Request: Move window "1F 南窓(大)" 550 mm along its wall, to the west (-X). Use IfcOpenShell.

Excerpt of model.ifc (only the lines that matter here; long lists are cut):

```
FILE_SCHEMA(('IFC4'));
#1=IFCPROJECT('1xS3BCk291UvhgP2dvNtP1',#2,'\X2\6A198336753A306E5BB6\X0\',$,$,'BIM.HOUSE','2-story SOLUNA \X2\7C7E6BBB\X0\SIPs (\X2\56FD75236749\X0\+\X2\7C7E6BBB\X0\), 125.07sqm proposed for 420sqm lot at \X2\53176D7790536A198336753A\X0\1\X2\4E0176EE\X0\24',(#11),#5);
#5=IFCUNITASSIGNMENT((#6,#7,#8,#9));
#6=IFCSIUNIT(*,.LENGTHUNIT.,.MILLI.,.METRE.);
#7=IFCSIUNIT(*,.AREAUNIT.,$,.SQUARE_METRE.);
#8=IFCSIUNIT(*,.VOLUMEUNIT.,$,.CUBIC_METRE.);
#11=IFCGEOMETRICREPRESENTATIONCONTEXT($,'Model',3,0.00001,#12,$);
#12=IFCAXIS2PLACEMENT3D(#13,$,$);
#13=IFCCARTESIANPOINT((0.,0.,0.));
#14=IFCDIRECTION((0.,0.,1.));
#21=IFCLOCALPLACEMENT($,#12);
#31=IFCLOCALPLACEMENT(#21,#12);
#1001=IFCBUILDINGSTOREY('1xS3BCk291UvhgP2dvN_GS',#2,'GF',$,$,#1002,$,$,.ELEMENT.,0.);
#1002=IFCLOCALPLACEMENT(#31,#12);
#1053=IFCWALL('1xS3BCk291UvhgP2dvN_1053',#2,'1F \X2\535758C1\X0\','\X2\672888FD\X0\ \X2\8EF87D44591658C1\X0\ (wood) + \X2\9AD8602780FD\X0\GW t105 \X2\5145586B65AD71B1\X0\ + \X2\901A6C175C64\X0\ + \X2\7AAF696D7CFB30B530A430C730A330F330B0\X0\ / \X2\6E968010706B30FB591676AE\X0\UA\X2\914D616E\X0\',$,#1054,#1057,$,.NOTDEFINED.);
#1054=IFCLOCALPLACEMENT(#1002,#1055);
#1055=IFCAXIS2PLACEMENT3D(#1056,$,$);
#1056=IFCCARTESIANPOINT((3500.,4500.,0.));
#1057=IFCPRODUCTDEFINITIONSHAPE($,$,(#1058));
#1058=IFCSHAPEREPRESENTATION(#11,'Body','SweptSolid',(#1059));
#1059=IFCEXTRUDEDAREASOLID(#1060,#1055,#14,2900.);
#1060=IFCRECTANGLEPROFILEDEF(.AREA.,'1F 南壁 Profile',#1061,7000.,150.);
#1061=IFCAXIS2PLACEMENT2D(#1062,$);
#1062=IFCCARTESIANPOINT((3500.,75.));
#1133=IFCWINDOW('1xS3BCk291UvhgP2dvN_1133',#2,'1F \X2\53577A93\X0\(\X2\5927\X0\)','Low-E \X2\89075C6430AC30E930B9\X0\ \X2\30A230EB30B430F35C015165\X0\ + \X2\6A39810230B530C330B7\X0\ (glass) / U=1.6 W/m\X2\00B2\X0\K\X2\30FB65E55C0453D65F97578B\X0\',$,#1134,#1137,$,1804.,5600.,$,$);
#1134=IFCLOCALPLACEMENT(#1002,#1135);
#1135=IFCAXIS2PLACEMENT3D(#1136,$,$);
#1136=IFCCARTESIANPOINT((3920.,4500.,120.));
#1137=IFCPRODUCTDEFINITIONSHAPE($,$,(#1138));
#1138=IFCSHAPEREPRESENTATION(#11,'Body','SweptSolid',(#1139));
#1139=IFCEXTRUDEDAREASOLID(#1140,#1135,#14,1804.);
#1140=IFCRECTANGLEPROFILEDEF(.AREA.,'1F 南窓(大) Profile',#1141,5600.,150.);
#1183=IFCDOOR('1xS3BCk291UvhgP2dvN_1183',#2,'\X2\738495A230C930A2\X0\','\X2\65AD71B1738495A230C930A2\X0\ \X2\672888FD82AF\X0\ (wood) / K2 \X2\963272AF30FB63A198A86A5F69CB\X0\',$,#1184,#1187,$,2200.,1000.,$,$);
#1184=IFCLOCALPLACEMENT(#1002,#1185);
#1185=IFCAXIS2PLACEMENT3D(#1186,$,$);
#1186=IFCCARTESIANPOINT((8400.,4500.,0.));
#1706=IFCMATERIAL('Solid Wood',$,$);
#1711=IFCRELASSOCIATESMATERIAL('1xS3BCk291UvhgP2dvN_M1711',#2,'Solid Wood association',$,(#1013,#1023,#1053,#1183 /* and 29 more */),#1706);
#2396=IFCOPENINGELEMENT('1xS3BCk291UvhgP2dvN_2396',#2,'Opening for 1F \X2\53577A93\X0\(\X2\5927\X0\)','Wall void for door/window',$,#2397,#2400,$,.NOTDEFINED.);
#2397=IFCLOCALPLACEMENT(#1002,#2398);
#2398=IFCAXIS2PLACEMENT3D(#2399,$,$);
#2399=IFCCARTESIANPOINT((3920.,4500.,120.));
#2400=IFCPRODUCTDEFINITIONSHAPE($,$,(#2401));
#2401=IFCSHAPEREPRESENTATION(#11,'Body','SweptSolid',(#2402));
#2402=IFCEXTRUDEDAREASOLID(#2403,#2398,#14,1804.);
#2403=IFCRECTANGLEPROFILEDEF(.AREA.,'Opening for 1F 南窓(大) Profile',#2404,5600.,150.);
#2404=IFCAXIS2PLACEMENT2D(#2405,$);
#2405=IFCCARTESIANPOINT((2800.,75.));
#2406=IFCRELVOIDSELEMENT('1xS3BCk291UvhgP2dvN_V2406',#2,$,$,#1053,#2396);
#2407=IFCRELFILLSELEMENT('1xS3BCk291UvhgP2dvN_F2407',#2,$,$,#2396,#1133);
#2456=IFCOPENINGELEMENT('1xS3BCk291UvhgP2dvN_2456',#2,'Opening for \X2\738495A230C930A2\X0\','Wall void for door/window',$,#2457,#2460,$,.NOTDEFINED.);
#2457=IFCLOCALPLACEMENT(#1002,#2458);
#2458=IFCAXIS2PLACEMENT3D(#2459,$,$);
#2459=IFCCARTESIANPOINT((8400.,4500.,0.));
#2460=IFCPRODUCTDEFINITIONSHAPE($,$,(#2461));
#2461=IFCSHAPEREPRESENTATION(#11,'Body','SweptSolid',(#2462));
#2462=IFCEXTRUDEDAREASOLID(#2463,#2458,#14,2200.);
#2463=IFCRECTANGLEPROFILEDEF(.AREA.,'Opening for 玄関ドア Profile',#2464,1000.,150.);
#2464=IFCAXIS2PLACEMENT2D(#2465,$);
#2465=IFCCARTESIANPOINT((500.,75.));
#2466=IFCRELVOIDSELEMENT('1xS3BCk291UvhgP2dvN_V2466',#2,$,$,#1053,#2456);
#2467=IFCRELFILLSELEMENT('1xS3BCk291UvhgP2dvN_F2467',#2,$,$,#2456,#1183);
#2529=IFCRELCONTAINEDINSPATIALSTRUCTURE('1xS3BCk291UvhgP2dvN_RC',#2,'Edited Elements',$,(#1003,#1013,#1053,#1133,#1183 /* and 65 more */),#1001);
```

```python
import ifcopenshell
import ifcopenshell.api.geometry
import ifcopenshell.util.placement
import ifcopenshell.util.unit

model = ifcopenshell.open("model.ifc")
unit_scale = ifcopenshell.util.unit.calculate_unit_scale(model)

window = model.by_guid("1xS3BCk291UvhgP2dvN_1133")
opening = window.FillsVoids[0].RelatingOpeningElement
wall = opening.VoidsElements[0].RelatingBuildingElement

wall_matrix = ifcopenshell.util.placement.get_local_placement(wall.ObjectPlacement)
shift = wall_matrix[:3, 0] * -0.55 / unit_scale
before = ifcopenshell.util.placement.get_local_placement(window.ObjectPlacement)[:3, 3].copy()

# The window is not placed relative to its opening, so move both.
for product in (opening, window):
    matrix = ifcopenshell.util.placement.get_local_placement(product.ObjectPlacement)
    matrix[:3, 3] += shift
    ifcopenshell.api.geometry.edit_object_placement(model, product=product, matrix=matrix, is_si=False)

after = ifcopenshell.util.placement.get_local_placement(window.ObjectPlacement)[:3, 3]
print("window moved by", (after - before).round(3) + 0.0)

model.write("model_updated.ifc")
```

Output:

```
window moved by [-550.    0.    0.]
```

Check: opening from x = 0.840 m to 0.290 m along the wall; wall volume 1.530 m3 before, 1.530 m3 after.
